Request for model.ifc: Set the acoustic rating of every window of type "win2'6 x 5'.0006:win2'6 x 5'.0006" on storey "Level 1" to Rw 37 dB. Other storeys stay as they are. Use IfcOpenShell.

First a look at what the model holds.

```python
import ifcopenshell
import ifcopenshell.util.element

model = ifcopenshell.open("model.ifc")
print(model.schema)
storey = next(s for s in model.by_type("IfcBuildingStorey") if s.Name == "Level 1")
windows = [e for e in ifcopenshell.util.element.get_decomposition(storey) if e.is_a("IfcWindow")]
seen = {}
for e in windows:
    element_type = ifcopenshell.util.element.get_type(e)
    key = (element_type.Name if element_type != e and element_type else None, ifcopenshell.util.element.get_pset(e, "Pset_WindowCommon", "AcousticRating"))
    seen[key] = seen.get(key, 0) + 1
for (name, value), count in sorted(seen.items(), key=str):
    print(count, "x", name, "|", value)
```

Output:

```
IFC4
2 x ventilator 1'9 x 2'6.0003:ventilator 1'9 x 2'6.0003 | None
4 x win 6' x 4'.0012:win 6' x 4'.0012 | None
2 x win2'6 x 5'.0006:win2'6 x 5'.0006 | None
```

```python
import ifcopenshell
import ifcopenshell.api.pset
import ifcopenshell.util.element

model = ifcopenshell.open("model.ifc")

storey = next(s for s in model.by_type("IfcBuildingStorey") if s.Name == "Level 1")
windows = [e for e in ifcopenshell.util.element.get_decomposition(storey) if e.is_a("IfcWindow")]

count = 0
for e in windows:
    element_type = ifcopenshell.util.element.get_type(e)
    if element_type in (None, e) or element_type.Name != "win2'6 x 5'.0006:win2'6 x 5'.0006":
        continue
    # add_pset returns the element's existing set when there is one.
    pset = ifcopenshell.api.pset.add_pset(model, product=e, name="Pset_WindowCommon")
    ifcopenshell.api.pset.edit_pset(model, pset=pset, properties={"AcousticRating": "Rw 37 dB"})
    count += 1

print(count, "windows updated")

model.write("model_v2.ifc")
```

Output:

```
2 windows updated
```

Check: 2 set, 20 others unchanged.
